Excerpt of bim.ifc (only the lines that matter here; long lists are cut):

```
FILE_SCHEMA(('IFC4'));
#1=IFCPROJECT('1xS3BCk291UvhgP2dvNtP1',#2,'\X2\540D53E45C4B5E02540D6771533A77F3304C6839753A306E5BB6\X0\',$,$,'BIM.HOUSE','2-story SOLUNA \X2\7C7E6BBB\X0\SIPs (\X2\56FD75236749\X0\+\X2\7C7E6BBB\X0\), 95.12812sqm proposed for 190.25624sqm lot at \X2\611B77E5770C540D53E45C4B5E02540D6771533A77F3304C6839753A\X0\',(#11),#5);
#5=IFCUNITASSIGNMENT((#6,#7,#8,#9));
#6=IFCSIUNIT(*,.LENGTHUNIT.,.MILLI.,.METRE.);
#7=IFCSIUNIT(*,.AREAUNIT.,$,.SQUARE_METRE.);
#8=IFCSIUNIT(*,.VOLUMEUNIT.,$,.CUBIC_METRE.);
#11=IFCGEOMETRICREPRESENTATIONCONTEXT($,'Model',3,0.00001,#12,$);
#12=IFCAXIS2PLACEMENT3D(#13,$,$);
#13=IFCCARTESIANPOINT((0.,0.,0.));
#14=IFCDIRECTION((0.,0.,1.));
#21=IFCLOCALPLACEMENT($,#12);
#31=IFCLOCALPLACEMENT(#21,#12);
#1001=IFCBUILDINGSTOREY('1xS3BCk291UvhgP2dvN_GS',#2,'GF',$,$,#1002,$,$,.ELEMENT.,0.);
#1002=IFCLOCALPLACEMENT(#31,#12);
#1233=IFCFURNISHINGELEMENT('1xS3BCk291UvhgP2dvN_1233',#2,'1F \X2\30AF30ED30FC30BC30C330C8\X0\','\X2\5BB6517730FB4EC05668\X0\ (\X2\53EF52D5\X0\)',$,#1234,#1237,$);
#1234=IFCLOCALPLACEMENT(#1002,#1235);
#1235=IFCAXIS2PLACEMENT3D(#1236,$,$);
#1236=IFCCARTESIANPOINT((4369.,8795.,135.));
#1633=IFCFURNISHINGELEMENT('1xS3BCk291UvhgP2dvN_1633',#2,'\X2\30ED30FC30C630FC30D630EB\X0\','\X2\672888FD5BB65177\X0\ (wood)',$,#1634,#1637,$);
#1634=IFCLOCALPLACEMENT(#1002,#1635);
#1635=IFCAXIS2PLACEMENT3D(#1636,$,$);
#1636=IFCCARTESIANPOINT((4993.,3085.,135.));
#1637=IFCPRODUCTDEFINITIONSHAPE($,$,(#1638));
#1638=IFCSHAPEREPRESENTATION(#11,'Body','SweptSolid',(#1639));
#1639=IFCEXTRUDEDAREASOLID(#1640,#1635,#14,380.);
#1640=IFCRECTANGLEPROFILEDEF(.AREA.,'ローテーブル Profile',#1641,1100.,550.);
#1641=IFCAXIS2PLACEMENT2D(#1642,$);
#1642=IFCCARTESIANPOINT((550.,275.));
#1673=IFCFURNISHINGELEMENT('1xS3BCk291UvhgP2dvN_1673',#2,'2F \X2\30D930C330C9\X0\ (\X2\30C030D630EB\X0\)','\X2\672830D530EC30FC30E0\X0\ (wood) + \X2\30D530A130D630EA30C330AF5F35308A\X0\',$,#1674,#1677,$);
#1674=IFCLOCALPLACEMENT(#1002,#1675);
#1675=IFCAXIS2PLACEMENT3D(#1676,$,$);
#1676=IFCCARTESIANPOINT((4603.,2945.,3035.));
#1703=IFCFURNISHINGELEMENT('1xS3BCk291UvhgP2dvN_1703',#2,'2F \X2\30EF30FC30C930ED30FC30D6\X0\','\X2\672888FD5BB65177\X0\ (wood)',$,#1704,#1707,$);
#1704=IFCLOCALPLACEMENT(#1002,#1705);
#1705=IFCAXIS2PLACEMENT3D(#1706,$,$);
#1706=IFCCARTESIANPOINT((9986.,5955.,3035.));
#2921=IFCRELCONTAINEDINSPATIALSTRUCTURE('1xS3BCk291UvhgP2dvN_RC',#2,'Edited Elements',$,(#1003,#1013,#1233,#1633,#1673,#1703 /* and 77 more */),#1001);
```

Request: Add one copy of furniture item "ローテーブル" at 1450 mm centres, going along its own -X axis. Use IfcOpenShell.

```python
import ifcopenshell
import ifcopenshell.api.geometry
import ifcopenshell.api.root
import ifcopenshell.util.element
import ifcopenshell.util.placement

model = ifcopenshell.open("bim.ifc")


def reuse_history(source, copy):
    """copy_class also copies each property set's owner history, people and application; keep the originals."""
    for rel in copy.IsDefinedBy:
        if rel.is_a("IfcRelDefinesByProperties") and (history := rel.RelatingPropertyDefinition.OwnerHistory):
            rel.RelatingPropertyDefinition.OwnerHistory = source.OwnerHistory
            ifcopenshell.util.element.remove_deep2(model, history)


source = model.by_guid("1xS3BCk291UvhgP2dvN_1633")
base = ifcopenshell.util.placement.get_local_placement(source.ObjectPlacement)
step = -base[:3, 0] * 1450.0

for i in range(1, 2):
    copy = ifcopenshell.api.root.copy_class(model, product=source)
    copy.Representation = ifcopenshell.util.element.copy_deep(
        model, source.Representation, exclude=["IfcGeometricRepresentationContext", "IfcRepresentationMap"]
    )
    reuse_history(source, copy)
    matrix = base.copy()
    matrix[:3, 3] += i * step
    print("added at", matrix[:3, 3].round(3) + 0.0)
    ifcopenshell.api.geometry.edit_object_placement(model, product=copy, matrix=matrix, is_si=False)

model.write("bim_edited.ifc")
```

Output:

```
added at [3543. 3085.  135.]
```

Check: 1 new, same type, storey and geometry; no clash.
